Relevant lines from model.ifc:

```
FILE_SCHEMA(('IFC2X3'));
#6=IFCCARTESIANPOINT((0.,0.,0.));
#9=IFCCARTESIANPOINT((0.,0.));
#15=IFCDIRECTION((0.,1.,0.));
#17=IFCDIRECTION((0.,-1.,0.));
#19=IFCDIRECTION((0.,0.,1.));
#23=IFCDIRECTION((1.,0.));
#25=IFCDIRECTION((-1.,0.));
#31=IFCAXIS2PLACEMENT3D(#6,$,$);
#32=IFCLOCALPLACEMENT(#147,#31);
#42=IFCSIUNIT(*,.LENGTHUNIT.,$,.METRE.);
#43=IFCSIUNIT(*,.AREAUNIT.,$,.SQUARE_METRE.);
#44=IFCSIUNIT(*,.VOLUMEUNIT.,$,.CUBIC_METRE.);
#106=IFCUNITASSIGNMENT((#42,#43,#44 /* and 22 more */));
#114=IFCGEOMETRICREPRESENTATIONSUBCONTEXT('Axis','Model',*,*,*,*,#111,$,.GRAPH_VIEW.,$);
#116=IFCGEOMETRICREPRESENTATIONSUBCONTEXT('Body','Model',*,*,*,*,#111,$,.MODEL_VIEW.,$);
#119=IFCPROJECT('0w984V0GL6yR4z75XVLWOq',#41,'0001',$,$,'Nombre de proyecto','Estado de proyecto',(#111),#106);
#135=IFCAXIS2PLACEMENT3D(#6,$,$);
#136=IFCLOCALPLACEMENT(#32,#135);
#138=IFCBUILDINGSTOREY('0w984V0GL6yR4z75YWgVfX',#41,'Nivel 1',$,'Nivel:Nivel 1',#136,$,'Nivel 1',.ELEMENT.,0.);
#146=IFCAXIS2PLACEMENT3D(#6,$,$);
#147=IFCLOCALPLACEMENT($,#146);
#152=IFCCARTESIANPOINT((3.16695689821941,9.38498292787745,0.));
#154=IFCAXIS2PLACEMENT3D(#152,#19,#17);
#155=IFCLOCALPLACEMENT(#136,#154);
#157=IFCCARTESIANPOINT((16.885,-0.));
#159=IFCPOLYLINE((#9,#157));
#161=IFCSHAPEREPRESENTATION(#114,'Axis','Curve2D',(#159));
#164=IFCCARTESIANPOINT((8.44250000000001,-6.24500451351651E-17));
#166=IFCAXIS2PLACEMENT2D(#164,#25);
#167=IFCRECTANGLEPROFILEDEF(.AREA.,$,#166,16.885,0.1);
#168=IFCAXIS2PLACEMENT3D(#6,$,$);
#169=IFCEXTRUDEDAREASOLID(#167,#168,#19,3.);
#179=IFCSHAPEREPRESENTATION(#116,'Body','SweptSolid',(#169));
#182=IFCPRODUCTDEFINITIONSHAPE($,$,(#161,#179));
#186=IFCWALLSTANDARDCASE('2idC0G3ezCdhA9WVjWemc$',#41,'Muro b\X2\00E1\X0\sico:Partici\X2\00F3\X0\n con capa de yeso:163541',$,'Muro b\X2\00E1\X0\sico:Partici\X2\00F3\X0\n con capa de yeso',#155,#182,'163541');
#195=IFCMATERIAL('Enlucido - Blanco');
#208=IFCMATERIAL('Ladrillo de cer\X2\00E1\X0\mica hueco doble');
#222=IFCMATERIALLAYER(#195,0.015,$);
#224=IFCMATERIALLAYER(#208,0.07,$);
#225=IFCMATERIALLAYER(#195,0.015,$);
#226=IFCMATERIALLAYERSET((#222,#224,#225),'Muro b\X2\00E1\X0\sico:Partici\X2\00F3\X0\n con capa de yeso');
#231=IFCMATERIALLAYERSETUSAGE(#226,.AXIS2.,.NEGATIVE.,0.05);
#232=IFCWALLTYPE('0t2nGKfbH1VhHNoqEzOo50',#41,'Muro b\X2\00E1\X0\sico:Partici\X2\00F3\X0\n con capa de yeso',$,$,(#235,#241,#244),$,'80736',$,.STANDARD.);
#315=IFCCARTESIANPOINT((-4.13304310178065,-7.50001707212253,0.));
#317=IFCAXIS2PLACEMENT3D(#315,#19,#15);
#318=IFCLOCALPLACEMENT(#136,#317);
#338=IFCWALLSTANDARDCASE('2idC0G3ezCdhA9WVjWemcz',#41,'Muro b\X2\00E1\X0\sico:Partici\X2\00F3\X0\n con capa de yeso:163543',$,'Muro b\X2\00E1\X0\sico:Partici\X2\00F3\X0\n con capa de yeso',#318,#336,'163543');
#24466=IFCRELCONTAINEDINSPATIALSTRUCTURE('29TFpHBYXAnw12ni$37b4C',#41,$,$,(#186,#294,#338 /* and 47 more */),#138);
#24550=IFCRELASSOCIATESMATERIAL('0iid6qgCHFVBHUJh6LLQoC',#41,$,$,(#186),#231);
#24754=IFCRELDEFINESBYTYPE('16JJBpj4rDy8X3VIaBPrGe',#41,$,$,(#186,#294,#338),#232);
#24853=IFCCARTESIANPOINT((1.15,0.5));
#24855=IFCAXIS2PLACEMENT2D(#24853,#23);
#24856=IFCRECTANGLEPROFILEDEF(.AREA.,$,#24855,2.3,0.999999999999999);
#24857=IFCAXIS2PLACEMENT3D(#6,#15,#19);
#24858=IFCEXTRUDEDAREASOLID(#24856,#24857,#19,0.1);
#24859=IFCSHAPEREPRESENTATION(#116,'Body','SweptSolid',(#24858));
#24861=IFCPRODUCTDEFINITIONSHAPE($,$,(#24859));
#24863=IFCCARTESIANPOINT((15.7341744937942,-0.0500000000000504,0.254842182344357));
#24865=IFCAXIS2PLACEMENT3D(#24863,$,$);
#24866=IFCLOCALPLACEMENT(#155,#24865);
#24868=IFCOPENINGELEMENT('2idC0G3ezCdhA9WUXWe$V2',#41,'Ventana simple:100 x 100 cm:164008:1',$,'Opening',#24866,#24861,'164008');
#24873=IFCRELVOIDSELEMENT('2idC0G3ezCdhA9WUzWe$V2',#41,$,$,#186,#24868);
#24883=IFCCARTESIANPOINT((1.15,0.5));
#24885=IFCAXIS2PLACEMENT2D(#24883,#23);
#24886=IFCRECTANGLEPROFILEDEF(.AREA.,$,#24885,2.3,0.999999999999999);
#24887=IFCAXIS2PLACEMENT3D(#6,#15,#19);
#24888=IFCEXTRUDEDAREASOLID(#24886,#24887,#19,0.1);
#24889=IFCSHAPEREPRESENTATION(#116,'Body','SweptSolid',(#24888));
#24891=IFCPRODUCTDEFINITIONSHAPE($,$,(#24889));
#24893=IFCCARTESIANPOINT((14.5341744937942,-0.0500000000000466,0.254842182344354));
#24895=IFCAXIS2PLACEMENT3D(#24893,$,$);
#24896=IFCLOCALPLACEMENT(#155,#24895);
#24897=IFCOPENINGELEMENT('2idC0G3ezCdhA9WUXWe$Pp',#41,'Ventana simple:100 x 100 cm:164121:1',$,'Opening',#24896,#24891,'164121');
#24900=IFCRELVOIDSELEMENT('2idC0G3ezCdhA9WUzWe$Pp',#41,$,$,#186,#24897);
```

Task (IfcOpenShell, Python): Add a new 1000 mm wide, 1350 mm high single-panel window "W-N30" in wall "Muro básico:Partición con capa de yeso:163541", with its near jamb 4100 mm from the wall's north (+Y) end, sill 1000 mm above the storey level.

```python
import numpy as np
import ifcopenshell
import ifcopenshell.api.feature
import ifcopenshell.api.geometry
import ifcopenshell.api.root
import ifcopenshell.api.spatial
import ifcopenshell.api.type
import ifcopenshell.geom
import ifcopenshell.util.element
import ifcopenshell.util.placement
import ifcopenshell.util.representation
import ifcopenshell.util.shape
import ifcopenshell.util.unit

model = ifcopenshell.open("model.ifc")
unit_scale = ifcopenshell.util.unit.calculate_unit_scale(model)
settings = ifcopenshell.geom.settings()


def volume(element):
    """Net volume in cubic metres, openings subtracted."""
    shape = ifcopenshell.geom.create_shape(settings, element)
    return ifcopenshell.util.shape.get_volume(shape.geometry)


wall = model.by_guid("2idC0G3ezCdhA9WVjWemc$")
storey = ifcopenshell.util.element.get_container(wall, ifc_class="IfcBuildingStorey")
context = ifcopenshell.util.representation.get_context(model, "Model", "Body", "MODEL_VIEW")
before = volume(wall)

width, height, from_end, sill = 1, 1.35, 4.1, 1  # metres

# The wall runs along its own X axis, and the end named is its -X end.
wall_shape = ifcopenshell.geom.create_shape(settings, wall)
x, y, z = ifcopenshell.util.shape.get_vertices(wall_shape.geometry).T
start = x.min() + from_end
face, thickness = float(y.min()), float(y.max() - y.min())
wall_matrix = ifcopenshell.util.placement.get_local_placement(wall.ObjectPlacement)
level = ifcopenshell.util.placement.get_local_placement(storey.ObjectPlacement)[2, 3]


def in_wall(x, y):
    """Placement at x, y metres in the wall's axes, at sill height."""
    matrix = wall_matrix.copy()
    matrix[:, 3] = wall_matrix @ np.array([x / unit_scale, y / unit_scale, 0.0, 1.0])
    matrix[2, 3] = level + sill / unit_scale
    return matrix


# Opening: a box that overshoots both wall faces by 50 mm.
opening = ifcopenshell.api.root.create_entity(model, ifc_class="IfcOpeningElement")
box = ifcopenshell.api.geometry.add_wall_representation(
    model, context=context, length=width, height=height, thickness=thickness + 0.1
)
ifcopenshell.api.geometry.assign_representation(model, product=opening, representation=box)
ifcopenshell.api.geometry.edit_object_placement(model, product=opening, matrix=in_wall(start, face - 0.05), is_si=False)
ifcopenshell.api.feature.add_feature(model, feature=opening, element=wall)

window = ifcopenshell.api.root.create_entity(model, ifc_class="IfcWindow", name="W-N30")
window.OverallWidth, window.OverallHeight = width / unit_scale, height / unit_scale
body = ifcopenshell.api.geometry.add_window_representation(
    model,
    context=context,
    overall_width=window.OverallWidth,
    overall_height=window.OverallHeight,
    partition_type="SINGLE_PANEL",
)
ifcopenshell.api.geometry.assign_representation(model, product=window, representation=body)
ifcopenshell.api.spatial.assign_container(model, products=[window], relating_structure=storey)
fills = ifcopenshell.api.feature.add_filling(model, opening=opening, element=window)
fills.OwnerHistory = window.OwnerHistory  # required in IFC2X3

# IFC2X3 keeps the operation on the window style.
style = ifcopenshell.api.root.create_entity(model, ifc_class="IfcWindowStyle", name="W-N30")
style.OperationType, style.ConstructionType = "SINGLE_PANEL", "NOTDEFINED"
style.ParameterTakesPrecedence = style.Sizeable = False
ifcopenshell.api.type.assign_type(model, related_objects=[window], relating_type=style)

# Centre the window in the wall's thickness.
ifcopenshell.api.geometry.edit_object_placement(model, product=window, matrix=in_wall(start, face), is_si=False)
window_shape = ifcopenshell.geom.create_shape(settings, window)
depth = ifcopenshell.util.shape.get_vertices(window_shape.geometry)[:, 1]
offset = face + thickness / 2 - (depth.min() + depth.max()) / 2
ifcopenshell.api.geometry.edit_object_placement(model, product=window, matrix=in_wall(start, offset), is_si=False)

after = volume(wall)

print(f"wall volume {before:.3f} -> {after:.3f} m3")

model.write("model_updated.ifc")
```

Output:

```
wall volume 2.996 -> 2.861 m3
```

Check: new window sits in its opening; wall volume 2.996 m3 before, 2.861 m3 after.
